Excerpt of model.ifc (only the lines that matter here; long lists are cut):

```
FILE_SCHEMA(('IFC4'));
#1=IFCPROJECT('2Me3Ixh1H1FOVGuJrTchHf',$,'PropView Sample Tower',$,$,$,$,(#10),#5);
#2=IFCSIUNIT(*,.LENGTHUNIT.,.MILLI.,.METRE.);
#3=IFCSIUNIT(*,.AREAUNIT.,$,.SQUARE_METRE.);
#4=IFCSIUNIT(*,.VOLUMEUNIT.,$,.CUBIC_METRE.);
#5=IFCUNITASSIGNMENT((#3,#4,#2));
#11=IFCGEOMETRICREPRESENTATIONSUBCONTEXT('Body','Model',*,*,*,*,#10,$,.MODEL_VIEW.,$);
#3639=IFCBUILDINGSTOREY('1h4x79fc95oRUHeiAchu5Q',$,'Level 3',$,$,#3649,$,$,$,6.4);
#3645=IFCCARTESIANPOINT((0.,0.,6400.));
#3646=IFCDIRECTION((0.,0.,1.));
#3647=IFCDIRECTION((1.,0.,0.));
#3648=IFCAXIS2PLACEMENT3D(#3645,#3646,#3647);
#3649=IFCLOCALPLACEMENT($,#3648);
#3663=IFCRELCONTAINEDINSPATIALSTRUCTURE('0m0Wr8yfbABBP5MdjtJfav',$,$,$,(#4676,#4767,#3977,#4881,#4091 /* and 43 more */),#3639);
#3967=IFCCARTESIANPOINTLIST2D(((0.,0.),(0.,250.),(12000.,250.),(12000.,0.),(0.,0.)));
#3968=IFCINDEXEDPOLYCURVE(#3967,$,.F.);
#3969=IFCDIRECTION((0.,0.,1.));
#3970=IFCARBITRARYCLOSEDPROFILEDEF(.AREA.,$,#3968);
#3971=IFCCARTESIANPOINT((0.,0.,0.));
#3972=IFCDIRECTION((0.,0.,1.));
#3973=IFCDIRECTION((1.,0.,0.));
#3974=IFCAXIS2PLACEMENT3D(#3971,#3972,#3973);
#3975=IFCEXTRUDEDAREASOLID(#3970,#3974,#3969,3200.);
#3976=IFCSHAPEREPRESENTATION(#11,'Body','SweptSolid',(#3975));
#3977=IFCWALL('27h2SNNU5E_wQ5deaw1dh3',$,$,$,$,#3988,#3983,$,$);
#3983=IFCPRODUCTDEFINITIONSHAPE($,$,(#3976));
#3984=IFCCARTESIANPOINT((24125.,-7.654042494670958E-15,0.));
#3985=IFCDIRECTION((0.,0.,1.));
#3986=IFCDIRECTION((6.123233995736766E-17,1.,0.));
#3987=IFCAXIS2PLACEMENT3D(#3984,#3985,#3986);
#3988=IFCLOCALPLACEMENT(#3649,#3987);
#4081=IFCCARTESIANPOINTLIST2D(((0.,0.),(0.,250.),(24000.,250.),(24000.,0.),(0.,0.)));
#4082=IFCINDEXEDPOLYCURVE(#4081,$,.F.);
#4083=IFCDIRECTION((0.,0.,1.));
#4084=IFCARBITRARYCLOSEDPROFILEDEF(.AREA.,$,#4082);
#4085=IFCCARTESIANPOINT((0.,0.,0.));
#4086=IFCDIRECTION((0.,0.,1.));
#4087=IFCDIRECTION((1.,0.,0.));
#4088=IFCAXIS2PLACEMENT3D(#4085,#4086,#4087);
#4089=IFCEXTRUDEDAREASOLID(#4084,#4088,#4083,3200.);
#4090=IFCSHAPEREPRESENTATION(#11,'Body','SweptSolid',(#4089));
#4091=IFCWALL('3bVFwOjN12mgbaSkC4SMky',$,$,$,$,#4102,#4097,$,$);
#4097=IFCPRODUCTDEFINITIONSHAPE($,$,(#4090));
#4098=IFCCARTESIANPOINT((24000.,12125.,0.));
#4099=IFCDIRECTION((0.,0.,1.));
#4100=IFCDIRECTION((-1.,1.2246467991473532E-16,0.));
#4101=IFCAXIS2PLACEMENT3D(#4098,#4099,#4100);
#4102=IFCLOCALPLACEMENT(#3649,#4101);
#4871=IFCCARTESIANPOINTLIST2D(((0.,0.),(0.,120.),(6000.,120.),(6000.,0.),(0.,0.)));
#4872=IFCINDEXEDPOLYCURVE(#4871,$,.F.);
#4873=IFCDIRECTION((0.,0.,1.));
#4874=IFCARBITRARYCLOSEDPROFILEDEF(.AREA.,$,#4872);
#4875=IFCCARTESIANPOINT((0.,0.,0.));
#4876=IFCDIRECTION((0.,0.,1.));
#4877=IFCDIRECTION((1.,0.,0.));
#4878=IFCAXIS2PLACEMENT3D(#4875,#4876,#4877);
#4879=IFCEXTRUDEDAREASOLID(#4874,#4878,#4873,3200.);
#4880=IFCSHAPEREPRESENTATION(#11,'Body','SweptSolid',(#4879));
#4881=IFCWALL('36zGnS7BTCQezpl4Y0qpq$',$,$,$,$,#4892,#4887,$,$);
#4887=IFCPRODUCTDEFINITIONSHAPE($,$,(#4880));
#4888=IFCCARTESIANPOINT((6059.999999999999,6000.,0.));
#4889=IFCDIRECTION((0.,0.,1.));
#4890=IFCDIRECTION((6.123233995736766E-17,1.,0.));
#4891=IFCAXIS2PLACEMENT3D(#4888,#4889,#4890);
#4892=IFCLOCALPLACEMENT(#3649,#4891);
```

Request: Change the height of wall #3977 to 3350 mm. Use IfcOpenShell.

```python
import ifcopenshell
import ifcopenshell.geom
import ifcopenshell.util.representation
import ifcopenshell.util.shape

model = ifcopenshell.open("model.ifc")
settings = ifcopenshell.geom.settings()


def volume(element):
    """Net volume in cubic metres, openings subtracted."""
    shape = ifcopenshell.geom.create_shape(settings, element)
    return ifcopenshell.util.shape.get_volume(shape.geometry)


wall = model.by_guid("27h2SNNU5E_wQ5deaw1dh3")
before = volume(wall)

body = ifcopenshell.util.representation.get_representation(wall, "Model", "Body")
solid = body.Items[0]
old_height = solid.Depth
solid.Depth = 3350.0
after = volume(wall)

print(f"height {old_height:g} -> {solid.Depth:g}, volume {before:.3f} -> {after:.3f} m3")

model.write("model_v2.ifc")
```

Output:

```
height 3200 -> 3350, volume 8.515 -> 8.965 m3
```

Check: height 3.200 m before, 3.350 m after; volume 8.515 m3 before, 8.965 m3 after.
